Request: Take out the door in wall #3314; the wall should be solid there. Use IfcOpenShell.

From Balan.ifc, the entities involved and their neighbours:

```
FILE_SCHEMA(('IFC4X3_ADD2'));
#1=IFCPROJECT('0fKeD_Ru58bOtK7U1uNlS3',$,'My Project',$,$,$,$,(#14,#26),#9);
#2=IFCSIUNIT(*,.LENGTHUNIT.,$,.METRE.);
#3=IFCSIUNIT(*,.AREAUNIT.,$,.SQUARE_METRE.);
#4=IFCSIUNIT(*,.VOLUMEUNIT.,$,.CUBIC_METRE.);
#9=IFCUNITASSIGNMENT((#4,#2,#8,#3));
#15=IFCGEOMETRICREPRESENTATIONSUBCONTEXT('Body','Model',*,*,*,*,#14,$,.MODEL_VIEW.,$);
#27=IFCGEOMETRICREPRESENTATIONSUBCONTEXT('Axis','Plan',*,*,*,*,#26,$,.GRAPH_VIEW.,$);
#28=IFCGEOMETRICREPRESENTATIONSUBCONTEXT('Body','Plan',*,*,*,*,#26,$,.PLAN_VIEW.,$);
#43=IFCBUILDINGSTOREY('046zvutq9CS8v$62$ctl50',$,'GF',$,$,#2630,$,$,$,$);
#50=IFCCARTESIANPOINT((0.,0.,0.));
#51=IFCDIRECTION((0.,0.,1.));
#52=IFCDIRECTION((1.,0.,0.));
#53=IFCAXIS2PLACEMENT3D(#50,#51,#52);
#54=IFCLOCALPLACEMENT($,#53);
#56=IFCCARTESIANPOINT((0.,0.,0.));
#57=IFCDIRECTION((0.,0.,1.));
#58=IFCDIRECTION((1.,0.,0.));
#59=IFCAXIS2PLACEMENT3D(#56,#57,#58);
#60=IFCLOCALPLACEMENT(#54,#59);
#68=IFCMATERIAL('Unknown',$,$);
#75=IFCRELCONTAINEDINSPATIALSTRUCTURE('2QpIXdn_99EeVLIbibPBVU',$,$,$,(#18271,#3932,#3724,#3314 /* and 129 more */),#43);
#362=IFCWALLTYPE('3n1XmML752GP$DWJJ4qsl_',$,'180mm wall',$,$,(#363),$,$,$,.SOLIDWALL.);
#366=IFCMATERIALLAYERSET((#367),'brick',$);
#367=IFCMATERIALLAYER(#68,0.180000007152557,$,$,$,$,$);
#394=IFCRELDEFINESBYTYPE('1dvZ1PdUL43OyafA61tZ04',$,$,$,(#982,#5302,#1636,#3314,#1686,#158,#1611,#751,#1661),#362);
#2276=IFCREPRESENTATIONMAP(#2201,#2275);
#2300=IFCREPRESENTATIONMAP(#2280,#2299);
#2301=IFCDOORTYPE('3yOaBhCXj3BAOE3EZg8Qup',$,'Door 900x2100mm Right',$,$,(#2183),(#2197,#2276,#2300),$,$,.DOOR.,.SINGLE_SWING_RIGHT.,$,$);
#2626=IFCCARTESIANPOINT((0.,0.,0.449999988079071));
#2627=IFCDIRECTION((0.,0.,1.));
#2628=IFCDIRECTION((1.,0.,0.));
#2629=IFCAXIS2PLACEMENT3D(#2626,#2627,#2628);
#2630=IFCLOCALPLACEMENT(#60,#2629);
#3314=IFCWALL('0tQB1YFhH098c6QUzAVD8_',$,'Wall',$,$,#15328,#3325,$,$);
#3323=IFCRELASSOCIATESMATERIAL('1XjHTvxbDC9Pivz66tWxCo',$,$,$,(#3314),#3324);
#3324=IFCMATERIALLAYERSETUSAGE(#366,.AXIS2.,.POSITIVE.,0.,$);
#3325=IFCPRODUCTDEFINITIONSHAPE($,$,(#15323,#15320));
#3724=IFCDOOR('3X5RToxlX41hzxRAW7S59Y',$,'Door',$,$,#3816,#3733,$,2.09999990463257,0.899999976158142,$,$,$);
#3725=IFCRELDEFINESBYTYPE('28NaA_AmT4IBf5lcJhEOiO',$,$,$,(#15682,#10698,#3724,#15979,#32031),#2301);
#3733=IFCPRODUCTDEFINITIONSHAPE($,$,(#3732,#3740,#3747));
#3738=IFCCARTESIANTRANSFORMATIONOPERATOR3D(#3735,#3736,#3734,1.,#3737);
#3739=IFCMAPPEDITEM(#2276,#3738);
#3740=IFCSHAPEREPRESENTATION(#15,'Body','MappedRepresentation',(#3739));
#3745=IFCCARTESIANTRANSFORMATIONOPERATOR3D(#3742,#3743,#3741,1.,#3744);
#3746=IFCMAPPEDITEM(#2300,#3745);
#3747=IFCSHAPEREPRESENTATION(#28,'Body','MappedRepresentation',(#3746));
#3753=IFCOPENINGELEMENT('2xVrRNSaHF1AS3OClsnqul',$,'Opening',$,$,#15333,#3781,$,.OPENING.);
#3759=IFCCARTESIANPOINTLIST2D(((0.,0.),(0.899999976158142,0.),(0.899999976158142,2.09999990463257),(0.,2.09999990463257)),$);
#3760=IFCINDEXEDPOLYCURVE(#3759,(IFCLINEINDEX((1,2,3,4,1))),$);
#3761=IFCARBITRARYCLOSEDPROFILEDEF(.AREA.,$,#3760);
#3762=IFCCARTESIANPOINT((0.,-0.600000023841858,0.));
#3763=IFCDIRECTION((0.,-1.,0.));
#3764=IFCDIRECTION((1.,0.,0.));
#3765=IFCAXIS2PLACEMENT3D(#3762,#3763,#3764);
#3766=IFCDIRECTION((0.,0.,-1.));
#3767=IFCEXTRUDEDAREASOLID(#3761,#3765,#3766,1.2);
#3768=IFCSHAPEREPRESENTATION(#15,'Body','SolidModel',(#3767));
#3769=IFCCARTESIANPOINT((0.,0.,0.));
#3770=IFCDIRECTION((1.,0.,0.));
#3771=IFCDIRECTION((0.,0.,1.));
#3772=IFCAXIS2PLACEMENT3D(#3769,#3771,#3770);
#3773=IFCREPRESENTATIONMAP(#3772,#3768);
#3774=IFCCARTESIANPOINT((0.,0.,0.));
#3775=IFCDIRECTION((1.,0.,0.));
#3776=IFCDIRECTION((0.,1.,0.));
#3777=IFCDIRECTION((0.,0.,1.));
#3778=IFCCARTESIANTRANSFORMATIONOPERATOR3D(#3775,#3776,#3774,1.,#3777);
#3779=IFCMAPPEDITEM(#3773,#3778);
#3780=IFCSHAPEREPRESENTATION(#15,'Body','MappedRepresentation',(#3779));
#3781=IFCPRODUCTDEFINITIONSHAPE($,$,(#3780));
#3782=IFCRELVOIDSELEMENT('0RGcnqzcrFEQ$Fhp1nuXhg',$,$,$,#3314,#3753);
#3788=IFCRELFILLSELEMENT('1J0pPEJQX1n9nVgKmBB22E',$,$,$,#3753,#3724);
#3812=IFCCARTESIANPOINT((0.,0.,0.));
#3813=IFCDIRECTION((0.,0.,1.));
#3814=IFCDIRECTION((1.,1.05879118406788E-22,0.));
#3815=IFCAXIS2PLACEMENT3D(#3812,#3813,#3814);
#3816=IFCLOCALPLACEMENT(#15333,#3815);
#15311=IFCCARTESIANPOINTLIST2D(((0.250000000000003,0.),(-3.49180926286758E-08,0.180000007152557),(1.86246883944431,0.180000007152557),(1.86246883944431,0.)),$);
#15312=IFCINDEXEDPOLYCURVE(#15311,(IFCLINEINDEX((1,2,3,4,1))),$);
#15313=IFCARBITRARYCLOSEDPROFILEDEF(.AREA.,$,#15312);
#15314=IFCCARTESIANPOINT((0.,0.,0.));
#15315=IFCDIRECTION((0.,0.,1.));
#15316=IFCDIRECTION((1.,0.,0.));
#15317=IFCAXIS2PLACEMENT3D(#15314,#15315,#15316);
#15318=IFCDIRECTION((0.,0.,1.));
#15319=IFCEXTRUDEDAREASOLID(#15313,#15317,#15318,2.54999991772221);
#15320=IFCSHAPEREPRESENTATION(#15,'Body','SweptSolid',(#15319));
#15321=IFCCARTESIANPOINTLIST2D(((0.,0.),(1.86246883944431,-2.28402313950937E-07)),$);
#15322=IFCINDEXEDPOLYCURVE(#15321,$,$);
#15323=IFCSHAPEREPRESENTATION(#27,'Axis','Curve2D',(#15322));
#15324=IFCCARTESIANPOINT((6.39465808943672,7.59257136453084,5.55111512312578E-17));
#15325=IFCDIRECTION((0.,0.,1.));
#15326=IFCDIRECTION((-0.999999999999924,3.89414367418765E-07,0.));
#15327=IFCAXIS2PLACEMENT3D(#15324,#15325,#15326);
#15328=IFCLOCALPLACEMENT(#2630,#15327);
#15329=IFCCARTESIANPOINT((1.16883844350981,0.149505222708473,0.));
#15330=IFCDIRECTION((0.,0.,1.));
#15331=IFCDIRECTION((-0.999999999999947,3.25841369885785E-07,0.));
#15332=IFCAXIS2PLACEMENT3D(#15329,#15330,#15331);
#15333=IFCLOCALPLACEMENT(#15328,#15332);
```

```python
import ifcopenshell
import ifcopenshell.api.feature
import ifcopenshell.api.root
import ifcopenshell.geom
import ifcopenshell.util.shape

model = ifcopenshell.open("Balan.ifc")
settings = ifcopenshell.geom.settings()


def volume(element):
    """Net volume in cubic metres, openings subtracted."""
    shape = ifcopenshell.geom.create_shape(settings, element)
    return ifcopenshell.util.shape.get_volume(shape.geometry)


door = model.by_guid("3X5RToxlX41hzxRAW7S59Y")
opening = door.FillsVoids[0].RelatingOpeningElement
wall = opening.VoidsElements[0].RelatingBuildingElement
before = volume(wall)

ifcopenshell.api.root.remove_product(model, product=door)
ifcopenshell.api.feature.remove_feature(model, feature=opening)

after = volume(wall)

print(f"wall volume {before:.3f} -> {after:.3f} m3")

model.write("Balan_v2.ifc")
```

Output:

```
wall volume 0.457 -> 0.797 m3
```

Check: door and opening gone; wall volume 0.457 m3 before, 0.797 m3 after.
